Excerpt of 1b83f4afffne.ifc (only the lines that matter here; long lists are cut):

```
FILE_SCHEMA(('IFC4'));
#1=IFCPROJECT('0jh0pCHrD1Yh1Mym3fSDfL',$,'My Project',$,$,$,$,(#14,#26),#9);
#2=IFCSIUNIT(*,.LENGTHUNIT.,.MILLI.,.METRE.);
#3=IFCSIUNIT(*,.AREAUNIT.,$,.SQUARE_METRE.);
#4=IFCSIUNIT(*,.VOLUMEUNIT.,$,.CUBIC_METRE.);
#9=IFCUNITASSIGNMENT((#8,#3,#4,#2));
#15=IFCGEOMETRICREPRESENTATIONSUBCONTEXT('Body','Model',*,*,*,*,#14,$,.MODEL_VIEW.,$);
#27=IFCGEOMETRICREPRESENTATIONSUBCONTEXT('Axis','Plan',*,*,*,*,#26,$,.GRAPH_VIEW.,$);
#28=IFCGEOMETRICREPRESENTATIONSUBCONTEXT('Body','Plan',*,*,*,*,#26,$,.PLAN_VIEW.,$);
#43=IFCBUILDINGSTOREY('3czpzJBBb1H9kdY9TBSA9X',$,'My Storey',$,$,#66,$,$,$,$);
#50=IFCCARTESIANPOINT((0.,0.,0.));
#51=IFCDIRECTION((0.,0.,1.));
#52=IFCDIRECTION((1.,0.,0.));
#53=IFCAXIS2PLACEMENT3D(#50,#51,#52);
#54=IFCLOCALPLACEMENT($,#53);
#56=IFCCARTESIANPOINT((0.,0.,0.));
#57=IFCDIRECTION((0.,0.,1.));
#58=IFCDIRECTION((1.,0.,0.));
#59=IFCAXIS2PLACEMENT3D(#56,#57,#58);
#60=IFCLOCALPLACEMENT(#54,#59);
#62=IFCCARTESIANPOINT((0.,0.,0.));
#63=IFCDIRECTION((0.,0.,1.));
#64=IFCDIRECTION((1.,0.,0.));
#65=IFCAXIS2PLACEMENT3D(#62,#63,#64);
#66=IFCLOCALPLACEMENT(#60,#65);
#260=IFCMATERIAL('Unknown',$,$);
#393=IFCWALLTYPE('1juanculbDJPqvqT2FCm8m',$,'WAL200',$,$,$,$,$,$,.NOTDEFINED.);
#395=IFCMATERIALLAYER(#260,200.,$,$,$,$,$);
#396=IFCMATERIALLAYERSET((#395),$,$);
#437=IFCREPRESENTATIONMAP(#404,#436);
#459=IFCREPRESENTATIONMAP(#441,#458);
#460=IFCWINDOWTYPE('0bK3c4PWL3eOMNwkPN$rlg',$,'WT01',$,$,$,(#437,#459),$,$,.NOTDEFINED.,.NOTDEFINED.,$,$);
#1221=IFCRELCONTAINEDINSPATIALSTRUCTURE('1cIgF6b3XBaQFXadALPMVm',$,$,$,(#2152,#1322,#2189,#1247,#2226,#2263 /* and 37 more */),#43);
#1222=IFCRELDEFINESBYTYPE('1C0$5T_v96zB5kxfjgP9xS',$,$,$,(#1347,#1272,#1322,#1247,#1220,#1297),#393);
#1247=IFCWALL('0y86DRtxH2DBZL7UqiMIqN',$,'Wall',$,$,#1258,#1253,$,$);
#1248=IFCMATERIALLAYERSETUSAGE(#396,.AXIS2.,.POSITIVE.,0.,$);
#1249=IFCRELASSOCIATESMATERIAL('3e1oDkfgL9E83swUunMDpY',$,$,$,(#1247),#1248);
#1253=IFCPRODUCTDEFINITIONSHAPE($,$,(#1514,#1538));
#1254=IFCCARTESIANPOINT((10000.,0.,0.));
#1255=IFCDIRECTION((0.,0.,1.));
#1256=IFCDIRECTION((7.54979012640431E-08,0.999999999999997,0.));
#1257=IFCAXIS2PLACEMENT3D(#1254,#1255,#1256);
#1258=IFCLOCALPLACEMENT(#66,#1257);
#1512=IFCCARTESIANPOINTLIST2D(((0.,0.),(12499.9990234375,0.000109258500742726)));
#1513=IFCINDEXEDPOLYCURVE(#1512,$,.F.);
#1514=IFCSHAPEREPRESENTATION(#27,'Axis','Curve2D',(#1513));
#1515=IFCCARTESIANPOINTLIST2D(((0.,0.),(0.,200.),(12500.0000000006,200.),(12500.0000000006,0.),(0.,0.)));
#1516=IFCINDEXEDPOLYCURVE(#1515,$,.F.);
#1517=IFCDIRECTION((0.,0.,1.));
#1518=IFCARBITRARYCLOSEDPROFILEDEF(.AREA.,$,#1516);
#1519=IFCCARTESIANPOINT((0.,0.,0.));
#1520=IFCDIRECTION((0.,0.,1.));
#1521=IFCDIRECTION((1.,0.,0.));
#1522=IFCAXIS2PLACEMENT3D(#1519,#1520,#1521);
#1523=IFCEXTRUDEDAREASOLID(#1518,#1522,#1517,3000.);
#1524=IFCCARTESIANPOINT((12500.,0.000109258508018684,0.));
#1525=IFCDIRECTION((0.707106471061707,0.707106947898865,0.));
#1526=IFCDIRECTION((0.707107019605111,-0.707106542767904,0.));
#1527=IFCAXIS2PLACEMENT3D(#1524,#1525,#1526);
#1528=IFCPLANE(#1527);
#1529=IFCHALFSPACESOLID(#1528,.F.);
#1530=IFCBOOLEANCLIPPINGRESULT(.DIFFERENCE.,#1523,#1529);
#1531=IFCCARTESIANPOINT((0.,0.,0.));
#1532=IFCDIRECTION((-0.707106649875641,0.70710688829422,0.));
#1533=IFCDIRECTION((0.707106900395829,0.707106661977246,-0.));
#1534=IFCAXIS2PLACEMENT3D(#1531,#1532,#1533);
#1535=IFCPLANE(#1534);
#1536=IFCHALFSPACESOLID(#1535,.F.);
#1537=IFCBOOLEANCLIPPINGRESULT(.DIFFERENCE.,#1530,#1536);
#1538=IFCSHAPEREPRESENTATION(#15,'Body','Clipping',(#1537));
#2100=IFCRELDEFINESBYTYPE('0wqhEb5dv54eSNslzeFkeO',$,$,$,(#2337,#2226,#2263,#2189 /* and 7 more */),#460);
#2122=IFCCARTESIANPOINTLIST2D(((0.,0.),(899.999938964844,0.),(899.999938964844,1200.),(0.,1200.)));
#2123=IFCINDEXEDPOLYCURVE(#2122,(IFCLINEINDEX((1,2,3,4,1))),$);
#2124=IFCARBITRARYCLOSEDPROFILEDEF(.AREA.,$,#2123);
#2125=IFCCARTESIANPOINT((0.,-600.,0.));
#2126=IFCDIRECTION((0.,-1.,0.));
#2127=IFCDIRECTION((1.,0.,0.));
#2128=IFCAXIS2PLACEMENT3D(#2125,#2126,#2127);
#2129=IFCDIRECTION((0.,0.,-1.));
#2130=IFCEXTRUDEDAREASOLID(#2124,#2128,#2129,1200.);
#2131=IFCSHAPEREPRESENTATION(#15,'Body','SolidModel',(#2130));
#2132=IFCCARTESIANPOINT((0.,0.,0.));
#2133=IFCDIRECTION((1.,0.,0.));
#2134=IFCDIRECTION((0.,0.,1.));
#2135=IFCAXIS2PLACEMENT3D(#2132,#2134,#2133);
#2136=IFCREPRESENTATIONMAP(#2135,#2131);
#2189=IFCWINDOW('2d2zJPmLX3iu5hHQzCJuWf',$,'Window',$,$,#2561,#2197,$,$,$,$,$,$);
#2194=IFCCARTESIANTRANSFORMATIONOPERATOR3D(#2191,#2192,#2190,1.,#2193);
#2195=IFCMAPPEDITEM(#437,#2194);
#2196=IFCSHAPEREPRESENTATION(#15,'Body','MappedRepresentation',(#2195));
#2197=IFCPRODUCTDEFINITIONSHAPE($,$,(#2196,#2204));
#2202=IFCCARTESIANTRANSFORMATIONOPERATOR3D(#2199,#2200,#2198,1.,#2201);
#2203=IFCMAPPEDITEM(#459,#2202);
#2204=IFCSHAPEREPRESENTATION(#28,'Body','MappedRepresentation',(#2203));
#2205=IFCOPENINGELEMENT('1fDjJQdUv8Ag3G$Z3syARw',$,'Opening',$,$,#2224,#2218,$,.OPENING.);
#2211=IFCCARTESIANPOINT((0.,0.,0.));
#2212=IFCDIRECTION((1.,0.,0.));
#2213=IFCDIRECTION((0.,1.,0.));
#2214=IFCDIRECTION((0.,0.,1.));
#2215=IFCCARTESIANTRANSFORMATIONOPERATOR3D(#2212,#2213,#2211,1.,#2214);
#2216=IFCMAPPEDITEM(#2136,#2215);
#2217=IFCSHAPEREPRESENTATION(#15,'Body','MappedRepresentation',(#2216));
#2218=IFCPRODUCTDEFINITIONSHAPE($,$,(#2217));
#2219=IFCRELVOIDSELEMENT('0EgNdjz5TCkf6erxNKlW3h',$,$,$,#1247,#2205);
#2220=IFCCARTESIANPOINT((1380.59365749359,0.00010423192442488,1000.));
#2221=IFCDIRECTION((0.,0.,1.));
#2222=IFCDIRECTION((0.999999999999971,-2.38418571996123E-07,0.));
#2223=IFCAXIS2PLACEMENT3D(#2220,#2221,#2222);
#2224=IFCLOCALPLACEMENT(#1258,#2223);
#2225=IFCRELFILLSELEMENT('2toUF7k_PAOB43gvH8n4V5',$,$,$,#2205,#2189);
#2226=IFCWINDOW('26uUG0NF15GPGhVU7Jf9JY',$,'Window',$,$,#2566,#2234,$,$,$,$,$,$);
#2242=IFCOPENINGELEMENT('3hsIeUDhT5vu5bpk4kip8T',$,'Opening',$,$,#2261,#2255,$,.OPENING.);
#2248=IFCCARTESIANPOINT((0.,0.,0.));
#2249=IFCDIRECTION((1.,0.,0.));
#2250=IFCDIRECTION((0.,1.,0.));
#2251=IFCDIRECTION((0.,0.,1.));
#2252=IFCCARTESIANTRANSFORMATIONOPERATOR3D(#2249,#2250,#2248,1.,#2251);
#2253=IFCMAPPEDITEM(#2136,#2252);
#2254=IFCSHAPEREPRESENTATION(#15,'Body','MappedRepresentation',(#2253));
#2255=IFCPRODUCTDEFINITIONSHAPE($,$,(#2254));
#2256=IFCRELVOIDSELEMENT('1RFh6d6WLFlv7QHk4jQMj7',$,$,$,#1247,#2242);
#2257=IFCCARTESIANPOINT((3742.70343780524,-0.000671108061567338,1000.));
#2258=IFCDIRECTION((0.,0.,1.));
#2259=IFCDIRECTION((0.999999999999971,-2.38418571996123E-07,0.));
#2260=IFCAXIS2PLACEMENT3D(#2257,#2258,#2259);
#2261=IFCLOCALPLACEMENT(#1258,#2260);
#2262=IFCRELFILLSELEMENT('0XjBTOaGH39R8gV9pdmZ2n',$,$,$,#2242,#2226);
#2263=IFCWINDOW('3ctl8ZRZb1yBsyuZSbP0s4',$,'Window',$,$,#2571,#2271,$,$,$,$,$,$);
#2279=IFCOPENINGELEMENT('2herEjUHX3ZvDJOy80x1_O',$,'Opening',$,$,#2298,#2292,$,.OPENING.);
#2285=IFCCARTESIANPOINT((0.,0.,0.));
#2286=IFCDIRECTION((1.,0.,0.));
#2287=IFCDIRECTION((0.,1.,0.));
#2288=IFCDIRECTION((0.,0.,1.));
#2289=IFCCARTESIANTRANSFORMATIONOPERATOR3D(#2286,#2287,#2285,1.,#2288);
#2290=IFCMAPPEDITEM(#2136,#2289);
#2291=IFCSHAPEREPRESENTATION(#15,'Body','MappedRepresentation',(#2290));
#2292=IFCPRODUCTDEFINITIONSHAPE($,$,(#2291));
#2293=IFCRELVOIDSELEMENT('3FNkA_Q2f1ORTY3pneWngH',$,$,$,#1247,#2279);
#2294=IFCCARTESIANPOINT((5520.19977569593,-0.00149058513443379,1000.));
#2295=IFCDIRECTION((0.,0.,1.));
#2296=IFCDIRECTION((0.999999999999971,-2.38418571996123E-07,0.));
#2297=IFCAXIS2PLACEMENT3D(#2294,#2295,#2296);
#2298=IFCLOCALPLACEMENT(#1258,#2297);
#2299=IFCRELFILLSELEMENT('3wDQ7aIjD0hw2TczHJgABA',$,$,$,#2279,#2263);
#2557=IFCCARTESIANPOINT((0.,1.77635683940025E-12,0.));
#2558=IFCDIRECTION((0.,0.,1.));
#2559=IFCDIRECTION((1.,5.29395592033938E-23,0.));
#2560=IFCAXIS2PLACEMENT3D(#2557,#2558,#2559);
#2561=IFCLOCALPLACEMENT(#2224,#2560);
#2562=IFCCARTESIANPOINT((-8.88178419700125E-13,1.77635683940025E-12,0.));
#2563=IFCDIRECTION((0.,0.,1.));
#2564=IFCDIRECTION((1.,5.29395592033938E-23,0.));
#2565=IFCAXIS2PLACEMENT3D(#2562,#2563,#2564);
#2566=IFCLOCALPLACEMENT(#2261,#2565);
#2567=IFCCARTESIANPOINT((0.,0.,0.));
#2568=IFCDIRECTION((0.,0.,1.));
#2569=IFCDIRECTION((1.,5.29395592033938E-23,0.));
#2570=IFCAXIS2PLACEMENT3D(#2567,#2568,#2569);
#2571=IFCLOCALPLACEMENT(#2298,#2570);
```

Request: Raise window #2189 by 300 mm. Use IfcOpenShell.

```python
import numpy as np
import ifcopenshell
import ifcopenshell.api.geometry
import ifcopenshell.util.placement
import ifcopenshell.util.unit

model = ifcopenshell.open("1b83f4afffne.ifc")
unit_scale = ifcopenshell.util.unit.calculate_unit_scale(model)

window = model.by_guid("2d2zJPmLX3iu5hHQzCJuWf")
opening = window.FillsVoids[0].RelatingOpeningElement
dz = 300.0

shift = np.array([0.0, 0.0, dz])
# The window is placed relative to its opening, so it follows when the opening moves.
matrix = ifcopenshell.util.placement.get_local_placement(opening.ObjectPlacement)
matrix[:3, 3] += shift
ifcopenshell.api.geometry.edit_object_placement(
    model, product=opening, matrix=matrix, is_si=False, should_transform_children=True
)

print(f"moved by {dz * unit_scale:+.3f} m")

model.write("1b83f4afffne_rev.ifc")
```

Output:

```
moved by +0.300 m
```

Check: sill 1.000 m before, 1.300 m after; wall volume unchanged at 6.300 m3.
